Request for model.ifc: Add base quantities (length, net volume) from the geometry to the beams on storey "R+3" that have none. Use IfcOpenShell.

First a look at what the model holds.

```python
import ifcopenshell
import ifcopenshell.util.element
import ifcopenshell.util.unit

model = ifcopenshell.open("model.ifc")
print(model.schema)
for unit_type in ("LENGTHUNIT", "AREAUNIT", "VOLUMEUNIT"):
    print(unit_type, ifcopenshell.util.unit.calculate_unit_scale(model, unit_type))
storey = next(s for s in model.by_type("IfcBuildingStorey") if s.Name == "R+3")
beams = [e for e in ifcopenshell.util.element.get_decomposition(storey) if e.is_a("IfcBeam")]
for e in sorted(beams, key=lambda e: e.id()):
    print(e.id(), e.is_a(), e.Name, list(ifcopenshell.util.element.get_psets(e, qtos_only=True)), sep=" | ")
```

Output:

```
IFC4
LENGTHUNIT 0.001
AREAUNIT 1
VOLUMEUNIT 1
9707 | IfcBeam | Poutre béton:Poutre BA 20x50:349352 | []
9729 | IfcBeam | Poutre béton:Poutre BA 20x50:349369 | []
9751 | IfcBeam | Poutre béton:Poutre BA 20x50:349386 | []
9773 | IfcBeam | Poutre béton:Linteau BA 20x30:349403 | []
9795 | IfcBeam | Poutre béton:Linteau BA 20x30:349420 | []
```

```python
import ifcopenshell
import ifcopenshell.api.pset
import ifcopenshell.geom
import ifcopenshell.util.element
import ifcopenshell.util.shape
import ifcopenshell.util.unit

model = ifcopenshell.open("model.ifc")
unit_scale = ifcopenshell.util.unit.calculate_unit_scale(model)
volume_scale = ifcopenshell.util.unit.calculate_unit_scale(model, "VOLUMEUNIT")
settings = ifcopenshell.geom.settings()

storey = next(s for s in model.by_type("IfcBuildingStorey") if s.Name == "R+3")
beams = [e for e in ifcopenshell.util.element.get_decomposition(storey) if e.is_a("IfcBeam")]

for e in sorted(beams, key=lambda e: e.id()):
    if ifcopenshell.util.element.get_psets(e, qtos_only=True, should_inherit=False):
        continue
    # Geometry comes back in metres, in the element's own axes.
    shape = ifcopenshell.geom.create_shape(settings, e)
    values = {
        "Length": ifcopenshell.util.shape.get_max_xyz(shape.geometry) / unit_scale,
        "NetVolume": ifcopenshell.util.shape.get_volume(shape.geometry) / volume_scale,
    }
    qto = ifcopenshell.api.pset.add_qto(model, product=e, name="Qto_BeamBaseQuantities")
    ifcopenshell.api.pset.edit_qto(model, qto=qto, properties=values)
    print(e.id(), {k: round(v, 3) for k, v in values.items()})

model.write("model_updated.ifc")
```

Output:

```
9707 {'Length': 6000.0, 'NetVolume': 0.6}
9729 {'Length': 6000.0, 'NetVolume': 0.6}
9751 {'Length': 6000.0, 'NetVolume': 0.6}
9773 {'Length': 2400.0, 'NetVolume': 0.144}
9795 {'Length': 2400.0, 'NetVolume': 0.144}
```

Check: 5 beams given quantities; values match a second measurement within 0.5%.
